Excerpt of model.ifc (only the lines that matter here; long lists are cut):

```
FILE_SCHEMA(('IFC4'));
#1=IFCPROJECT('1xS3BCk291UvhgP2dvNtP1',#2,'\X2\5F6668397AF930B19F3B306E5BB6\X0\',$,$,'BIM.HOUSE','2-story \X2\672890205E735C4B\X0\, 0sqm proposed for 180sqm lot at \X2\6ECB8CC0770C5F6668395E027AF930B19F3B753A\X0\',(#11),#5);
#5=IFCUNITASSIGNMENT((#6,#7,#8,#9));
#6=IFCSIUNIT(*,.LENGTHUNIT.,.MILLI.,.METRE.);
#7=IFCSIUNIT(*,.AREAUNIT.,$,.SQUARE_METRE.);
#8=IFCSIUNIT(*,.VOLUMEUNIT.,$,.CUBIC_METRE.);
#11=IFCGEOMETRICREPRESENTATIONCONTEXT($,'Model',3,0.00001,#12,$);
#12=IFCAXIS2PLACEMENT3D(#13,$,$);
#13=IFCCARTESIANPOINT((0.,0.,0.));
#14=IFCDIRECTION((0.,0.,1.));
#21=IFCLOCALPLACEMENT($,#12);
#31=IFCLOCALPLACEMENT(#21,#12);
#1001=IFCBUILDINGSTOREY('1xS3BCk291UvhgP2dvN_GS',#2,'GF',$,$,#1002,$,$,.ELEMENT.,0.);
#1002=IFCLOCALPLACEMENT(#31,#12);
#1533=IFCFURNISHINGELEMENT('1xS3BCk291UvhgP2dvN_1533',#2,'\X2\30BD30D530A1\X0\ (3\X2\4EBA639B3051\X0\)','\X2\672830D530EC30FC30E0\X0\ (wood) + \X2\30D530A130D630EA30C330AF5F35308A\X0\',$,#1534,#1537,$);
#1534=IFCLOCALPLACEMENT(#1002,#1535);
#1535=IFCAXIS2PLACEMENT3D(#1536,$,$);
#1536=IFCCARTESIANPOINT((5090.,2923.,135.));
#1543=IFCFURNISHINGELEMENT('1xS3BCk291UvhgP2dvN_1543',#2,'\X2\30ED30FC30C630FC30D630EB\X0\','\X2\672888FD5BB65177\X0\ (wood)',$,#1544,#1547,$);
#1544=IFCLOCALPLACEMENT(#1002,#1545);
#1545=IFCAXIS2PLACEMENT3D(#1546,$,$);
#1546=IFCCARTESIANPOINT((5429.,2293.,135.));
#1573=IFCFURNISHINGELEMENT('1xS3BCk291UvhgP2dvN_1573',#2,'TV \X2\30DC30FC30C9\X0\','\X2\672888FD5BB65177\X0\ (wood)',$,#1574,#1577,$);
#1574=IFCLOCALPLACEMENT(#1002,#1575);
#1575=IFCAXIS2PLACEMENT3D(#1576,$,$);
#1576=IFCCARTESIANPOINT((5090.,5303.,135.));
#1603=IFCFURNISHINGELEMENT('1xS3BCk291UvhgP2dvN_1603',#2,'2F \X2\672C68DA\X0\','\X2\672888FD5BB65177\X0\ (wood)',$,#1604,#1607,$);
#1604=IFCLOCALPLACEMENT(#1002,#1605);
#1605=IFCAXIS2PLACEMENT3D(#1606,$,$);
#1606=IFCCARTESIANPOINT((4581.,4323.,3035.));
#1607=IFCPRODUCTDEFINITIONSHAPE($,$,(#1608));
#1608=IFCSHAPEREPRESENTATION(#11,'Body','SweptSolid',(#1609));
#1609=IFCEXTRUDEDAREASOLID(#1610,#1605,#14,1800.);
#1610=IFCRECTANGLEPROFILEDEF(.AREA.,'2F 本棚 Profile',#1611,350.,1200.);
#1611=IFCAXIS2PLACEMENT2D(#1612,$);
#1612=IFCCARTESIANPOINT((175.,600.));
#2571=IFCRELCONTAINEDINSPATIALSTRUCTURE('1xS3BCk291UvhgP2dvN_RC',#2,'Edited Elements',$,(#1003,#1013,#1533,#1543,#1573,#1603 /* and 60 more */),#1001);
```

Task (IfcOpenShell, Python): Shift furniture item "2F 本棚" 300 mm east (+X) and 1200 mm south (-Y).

```python
import ifcopenshell
import ifcopenshell.api.geometry
import ifcopenshell.util.placement
import ifcopenshell.util.unit

model = ifcopenshell.open("model.ifc")
unit_scale = ifcopenshell.util.unit.calculate_unit_scale(model)

item = model.by_guid("1xS3BCk291UvhgP2dvN_1603")
matrix = ifcopenshell.util.placement.get_local_placement(item.ObjectPlacement)
matrix[0, 3] += 0.3 / unit_scale
matrix[1, 3] -= 1.2 / unit_scale
ifcopenshell.api.geometry.edit_object_placement(model, product=item, matrix=matrix, is_si=False)

print(ifcopenshell.util.placement.get_local_placement(item.ObjectPlacement).round(3) + 0.0)

model.write("model_updated.ifc")
```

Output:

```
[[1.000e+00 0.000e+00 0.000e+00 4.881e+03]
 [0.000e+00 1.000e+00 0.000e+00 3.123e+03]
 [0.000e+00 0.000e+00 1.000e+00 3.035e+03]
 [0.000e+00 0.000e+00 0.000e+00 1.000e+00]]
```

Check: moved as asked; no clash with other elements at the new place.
